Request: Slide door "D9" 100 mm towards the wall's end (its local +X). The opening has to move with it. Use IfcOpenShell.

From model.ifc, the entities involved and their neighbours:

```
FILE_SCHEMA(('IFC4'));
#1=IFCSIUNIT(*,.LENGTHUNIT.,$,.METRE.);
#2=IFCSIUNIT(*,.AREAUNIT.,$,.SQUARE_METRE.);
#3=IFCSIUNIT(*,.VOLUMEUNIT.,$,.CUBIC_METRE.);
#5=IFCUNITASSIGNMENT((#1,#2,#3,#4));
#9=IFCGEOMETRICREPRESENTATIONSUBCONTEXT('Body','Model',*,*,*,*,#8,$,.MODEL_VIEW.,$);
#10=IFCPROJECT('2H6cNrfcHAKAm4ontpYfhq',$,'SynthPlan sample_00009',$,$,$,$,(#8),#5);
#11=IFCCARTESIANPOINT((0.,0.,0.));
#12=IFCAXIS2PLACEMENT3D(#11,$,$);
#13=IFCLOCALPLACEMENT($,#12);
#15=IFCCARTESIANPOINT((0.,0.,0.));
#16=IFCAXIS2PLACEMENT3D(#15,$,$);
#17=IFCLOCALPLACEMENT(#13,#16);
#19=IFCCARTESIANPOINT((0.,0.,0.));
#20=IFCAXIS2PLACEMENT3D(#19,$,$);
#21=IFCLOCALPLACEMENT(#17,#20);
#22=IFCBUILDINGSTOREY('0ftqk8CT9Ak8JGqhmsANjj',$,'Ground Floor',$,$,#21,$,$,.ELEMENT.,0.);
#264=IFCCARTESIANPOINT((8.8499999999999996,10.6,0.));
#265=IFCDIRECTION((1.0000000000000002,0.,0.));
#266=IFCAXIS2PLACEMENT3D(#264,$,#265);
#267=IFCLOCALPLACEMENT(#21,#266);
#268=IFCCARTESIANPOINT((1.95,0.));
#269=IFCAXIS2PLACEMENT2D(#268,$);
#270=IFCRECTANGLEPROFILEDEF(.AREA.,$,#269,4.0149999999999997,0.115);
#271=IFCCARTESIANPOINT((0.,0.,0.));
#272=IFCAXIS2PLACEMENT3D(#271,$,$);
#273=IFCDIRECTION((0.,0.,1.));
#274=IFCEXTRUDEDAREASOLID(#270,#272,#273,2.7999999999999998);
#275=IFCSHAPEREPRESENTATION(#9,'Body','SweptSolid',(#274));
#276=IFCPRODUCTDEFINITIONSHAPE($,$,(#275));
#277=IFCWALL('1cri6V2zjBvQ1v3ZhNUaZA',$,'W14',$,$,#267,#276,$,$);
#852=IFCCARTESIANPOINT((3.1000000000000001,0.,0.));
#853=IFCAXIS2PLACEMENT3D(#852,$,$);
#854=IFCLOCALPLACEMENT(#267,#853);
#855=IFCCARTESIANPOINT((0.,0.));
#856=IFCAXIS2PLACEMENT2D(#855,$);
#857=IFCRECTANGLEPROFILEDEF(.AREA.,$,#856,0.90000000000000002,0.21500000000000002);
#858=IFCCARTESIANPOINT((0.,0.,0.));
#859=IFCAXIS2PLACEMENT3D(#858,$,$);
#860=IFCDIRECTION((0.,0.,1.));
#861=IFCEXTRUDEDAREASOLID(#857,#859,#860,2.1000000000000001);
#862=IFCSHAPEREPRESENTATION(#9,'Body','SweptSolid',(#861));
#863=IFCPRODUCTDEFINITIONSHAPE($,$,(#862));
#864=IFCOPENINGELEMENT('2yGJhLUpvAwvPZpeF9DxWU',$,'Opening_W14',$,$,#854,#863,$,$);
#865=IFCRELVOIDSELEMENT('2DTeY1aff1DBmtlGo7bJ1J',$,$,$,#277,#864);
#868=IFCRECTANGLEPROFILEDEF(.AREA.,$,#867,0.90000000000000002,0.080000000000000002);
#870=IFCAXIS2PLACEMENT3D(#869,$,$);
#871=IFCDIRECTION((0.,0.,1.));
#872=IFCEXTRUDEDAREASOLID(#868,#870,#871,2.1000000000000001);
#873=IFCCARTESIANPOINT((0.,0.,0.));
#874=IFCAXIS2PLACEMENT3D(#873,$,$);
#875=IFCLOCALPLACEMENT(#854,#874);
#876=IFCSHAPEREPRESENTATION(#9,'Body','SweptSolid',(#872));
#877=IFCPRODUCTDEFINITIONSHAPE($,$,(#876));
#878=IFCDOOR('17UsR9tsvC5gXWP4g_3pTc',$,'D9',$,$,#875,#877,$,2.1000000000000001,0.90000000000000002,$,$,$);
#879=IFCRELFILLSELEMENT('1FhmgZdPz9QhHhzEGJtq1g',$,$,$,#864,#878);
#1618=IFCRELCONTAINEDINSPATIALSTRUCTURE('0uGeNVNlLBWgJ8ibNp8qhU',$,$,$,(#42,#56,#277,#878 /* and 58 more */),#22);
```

```python
import ifcopenshell
import ifcopenshell.api.geometry
import ifcopenshell.util.placement

model = ifcopenshell.open("model.ifc")

door = model.by_id(878)
opening = door.FillsVoids[0].RelatingOpeningElement
wall = opening.VoidsElements[0].RelatingBuildingElement

wall_matrix = ifcopenshell.util.placement.get_local_placement(wall.ObjectPlacement)
shift = wall_matrix[:3, 0] * 0.1
before = ifcopenshell.util.placement.get_local_placement(door.ObjectPlacement)[:3, 3].copy()

# The door is placed relative to its opening, so it follows when the opening moves.
matrix = ifcopenshell.util.placement.get_local_placement(opening.ObjectPlacement)
matrix[:3, 3] += shift
ifcopenshell.api.geometry.edit_object_placement(
    model, product=opening, matrix=matrix, is_si=False, should_transform_children=True
)

after = ifcopenshell.util.placement.get_local_placement(door.ObjectPlacement)[:3, 3]
print("door moved by", (after - before).round(3) + 0.0)

model.write("model_rev.ifc")
```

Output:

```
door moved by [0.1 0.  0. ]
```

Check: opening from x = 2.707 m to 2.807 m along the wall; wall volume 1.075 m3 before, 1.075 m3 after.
